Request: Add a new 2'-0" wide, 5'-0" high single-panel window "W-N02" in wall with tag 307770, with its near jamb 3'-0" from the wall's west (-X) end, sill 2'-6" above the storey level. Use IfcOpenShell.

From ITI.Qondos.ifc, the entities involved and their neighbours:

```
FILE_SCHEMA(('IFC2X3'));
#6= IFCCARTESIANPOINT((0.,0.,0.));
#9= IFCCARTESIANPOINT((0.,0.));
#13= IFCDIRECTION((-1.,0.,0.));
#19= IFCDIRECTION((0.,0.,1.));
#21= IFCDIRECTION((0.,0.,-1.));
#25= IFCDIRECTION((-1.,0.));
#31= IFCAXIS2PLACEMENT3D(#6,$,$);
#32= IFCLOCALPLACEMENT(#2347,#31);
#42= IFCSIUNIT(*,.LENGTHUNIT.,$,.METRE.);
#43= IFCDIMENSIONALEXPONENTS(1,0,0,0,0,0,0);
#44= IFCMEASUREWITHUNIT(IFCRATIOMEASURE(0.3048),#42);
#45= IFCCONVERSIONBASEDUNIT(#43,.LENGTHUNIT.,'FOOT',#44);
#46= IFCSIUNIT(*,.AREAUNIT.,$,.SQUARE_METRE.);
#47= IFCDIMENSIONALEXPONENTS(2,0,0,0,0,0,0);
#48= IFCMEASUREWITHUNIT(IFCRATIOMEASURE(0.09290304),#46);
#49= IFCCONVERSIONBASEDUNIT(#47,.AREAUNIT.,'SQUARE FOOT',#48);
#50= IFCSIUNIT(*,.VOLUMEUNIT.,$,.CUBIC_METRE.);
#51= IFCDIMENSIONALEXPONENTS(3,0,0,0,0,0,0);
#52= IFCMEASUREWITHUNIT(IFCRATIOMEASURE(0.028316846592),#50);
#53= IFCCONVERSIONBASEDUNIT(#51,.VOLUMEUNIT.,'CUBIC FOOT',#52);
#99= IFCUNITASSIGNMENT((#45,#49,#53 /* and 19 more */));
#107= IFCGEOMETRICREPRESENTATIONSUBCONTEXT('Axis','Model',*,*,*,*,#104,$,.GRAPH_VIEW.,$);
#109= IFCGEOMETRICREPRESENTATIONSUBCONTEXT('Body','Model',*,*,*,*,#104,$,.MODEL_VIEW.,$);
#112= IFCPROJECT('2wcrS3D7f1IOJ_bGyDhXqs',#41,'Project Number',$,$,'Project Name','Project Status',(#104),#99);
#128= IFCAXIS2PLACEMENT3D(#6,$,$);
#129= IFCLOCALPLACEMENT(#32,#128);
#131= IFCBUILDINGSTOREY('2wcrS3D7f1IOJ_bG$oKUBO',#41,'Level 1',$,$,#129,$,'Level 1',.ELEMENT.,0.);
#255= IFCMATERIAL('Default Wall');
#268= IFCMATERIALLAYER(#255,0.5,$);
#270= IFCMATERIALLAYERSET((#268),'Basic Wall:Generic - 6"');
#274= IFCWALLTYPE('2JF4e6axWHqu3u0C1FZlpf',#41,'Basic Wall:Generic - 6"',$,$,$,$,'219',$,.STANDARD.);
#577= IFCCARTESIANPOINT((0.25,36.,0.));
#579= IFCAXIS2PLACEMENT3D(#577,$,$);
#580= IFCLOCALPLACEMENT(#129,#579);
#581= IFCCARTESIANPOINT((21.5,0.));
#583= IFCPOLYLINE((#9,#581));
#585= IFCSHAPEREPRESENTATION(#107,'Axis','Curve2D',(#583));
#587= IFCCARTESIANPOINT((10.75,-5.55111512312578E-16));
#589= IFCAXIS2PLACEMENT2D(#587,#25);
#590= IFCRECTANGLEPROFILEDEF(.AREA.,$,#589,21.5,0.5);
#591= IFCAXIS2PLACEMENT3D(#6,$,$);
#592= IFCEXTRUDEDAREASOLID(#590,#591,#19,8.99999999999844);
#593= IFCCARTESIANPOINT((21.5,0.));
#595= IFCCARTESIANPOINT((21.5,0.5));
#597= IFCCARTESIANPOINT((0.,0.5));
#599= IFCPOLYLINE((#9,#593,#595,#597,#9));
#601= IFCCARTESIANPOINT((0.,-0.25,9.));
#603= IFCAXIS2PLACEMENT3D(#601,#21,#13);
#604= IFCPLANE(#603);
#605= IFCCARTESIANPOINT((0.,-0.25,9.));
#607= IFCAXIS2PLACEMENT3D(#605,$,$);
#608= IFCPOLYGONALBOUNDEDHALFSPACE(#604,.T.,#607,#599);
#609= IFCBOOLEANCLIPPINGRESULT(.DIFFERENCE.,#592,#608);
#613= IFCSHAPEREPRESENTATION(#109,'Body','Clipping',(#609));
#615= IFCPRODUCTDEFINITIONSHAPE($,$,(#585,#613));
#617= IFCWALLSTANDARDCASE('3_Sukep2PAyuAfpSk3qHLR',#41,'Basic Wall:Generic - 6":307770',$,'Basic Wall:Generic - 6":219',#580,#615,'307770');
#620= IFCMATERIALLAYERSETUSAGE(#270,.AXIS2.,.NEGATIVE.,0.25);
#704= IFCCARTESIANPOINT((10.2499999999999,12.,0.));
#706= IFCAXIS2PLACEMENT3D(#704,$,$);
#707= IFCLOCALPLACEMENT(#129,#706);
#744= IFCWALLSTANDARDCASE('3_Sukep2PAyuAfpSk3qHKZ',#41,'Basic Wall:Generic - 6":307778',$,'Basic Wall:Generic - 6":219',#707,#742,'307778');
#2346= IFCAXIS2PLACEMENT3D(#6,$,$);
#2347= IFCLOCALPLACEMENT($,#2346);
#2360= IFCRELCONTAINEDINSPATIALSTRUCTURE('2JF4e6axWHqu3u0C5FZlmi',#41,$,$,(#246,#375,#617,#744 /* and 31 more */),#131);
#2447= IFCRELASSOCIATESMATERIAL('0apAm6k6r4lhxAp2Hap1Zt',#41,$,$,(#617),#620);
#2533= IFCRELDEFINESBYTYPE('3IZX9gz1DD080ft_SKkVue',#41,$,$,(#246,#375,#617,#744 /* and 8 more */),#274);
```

```python
import numpy as np
import ifcopenshell
import ifcopenshell.api.feature
import ifcopenshell.api.geometry
import ifcopenshell.api.root
import ifcopenshell.api.spatial
import ifcopenshell.api.type
import ifcopenshell.geom
import ifcopenshell.util.element
import ifcopenshell.util.placement
import ifcopenshell.util.representation
import ifcopenshell.util.shape
import ifcopenshell.util.unit

model = ifcopenshell.open("ITI.Qondos.ifc")
unit_scale = ifcopenshell.util.unit.calculate_unit_scale(model)
settings = ifcopenshell.geom.settings()


def volume(element):
    """Net volume in cubic metres, openings subtracted."""
    shape = ifcopenshell.geom.create_shape(settings, element)
    return ifcopenshell.util.shape.get_volume(shape.geometry)


wall = model.by_id(617)
storey = ifcopenshell.util.element.get_container(wall, ifc_class="IfcBuildingStorey")
context = ifcopenshell.util.representation.get_context(model, "Model", "Body", "MODEL_VIEW")
before = volume(wall)

width, height, from_end, sill = 0.6096, 1.524, 0.9144, 0.762  # metres

# The wall runs along its own X axis, and the end named is its -X end.
wall_shape = ifcopenshell.geom.create_shape(settings, wall)
x, y, z = ifcopenshell.util.shape.get_vertices(wall_shape.geometry).T
start = x.min() + from_end
face, thickness = float(y.min()), float(y.max() - y.min())
wall_matrix = ifcopenshell.util.placement.get_local_placement(wall.ObjectPlacement)
level = ifcopenshell.util.placement.get_local_placement(storey.ObjectPlacement)[2, 3]


def in_wall(x, y):
    """Placement at x, y metres in the wall's axes, at sill height."""
    matrix = wall_matrix.copy()
    matrix[:, 3] = wall_matrix @ np.array([x / unit_scale, y / unit_scale, 0.0, 1.0])
    matrix[2, 3] = level + sill / unit_scale
    return matrix


# Opening: a box that overshoots both wall faces by 50 mm.
opening = ifcopenshell.api.root.create_entity(model, ifc_class="IfcOpeningElement")
box = ifcopenshell.api.geometry.add_wall_representation(
    model, context=context, length=width, height=height, thickness=thickness + 0.1
)
ifcopenshell.api.geometry.assign_representation(model, product=opening, representation=box)
ifcopenshell.api.geometry.edit_object_placement(model, product=opening, matrix=in_wall(start, face - 0.05), is_si=False)
ifcopenshell.api.feature.add_feature(model, feature=opening, element=wall)

window = ifcopenshell.api.root.create_entity(model, ifc_class="IfcWindow", name="W-N02")
window.OverallWidth, window.OverallHeight = width / unit_scale, height / unit_scale
body = ifcopenshell.api.geometry.add_window_representation(
    model,
    context=context,
    overall_width=window.OverallWidth,
    overall_height=window.OverallHeight,
    partition_type="SINGLE_PANEL",
)
ifcopenshell.api.geometry.assign_representation(model, product=window, representation=body)
ifcopenshell.api.spatial.assign_container(model, products=[window], relating_structure=storey)
fills = ifcopenshell.api.feature.add_filling(model, opening=opening, element=window)
fills.OwnerHistory = window.OwnerHistory  # required in IFC2X3

# IFC2X3 keeps the operation on the window style.
style = ifcopenshell.api.root.create_entity(model, ifc_class="IfcWindowStyle", name="W-N02")
style.OperationType, style.ConstructionType = "SINGLE_PANEL", "NOTDEFINED"
style.ParameterTakesPrecedence = style.Sizeable = False
ifcopenshell.api.type.assign_type(model, related_objects=[window], relating_type=style)

# Centre the window in the wall's thickness.
ifcopenshell.api.geometry.edit_object_placement(model, product=window, matrix=in_wall(start, face), is_si=False)
window_shape = ifcopenshell.geom.create_shape(settings, window)
depth = ifcopenshell.util.shape.get_vertices(window_shape.geometry)[:, 1]
offset = face + thickness / 2 - (depth.min() + depth.max()) / 2
ifcopenshell.api.geometry.edit_object_placement(model, product=window, matrix=in_wall(start, offset), is_si=False)

after = volume(wall)

print(f"wall volume {before:.3f} -> {after:.3f} m3")

model.write("ITI.Qondos_v2.ifc")
```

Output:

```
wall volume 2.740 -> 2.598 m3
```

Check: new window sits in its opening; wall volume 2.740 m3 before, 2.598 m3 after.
